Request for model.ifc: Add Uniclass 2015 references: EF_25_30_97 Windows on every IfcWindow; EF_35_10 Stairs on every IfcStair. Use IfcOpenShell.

First a look at what the model holds.

```python
import ifcopenshell

model = ifcopenshell.open("model.ifc")
print(model.schema)
print("classifications:", [c.Name for c in model.by_type("IfcClassification")])
for ifc_class in ("IfcDoor", "IfcRoof", "IfcStair", "IfcWall", "IfcWindow"):
    print(ifc_class, len(model.by_type(ifc_class)))
```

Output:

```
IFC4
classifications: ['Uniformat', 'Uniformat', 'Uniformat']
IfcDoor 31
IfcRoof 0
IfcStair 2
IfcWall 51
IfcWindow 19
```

```python
import ifcopenshell
import ifcopenshell.api.classification

model = ifcopenshell.open("model.ifc")

system = ifcopenshell.api.classification.add_classification(model, classification="Uniclass 2015")

codes = {
    "IfcWindow": ("EF_25_30_97", "Windows"),
    "IfcStair": ("EF_35_10", "Stairs"),
}
for ifc_class, (code, name) in codes.items():
    products = model.by_type(ifc_class)
    ifcopenshell.api.classification.add_reference(
        model, products=products, classification=system, identification=code, name=name
    )
    print(code, len(products))

model.write("model_v2.ifc")
```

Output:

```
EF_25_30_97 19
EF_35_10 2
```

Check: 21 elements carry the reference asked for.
